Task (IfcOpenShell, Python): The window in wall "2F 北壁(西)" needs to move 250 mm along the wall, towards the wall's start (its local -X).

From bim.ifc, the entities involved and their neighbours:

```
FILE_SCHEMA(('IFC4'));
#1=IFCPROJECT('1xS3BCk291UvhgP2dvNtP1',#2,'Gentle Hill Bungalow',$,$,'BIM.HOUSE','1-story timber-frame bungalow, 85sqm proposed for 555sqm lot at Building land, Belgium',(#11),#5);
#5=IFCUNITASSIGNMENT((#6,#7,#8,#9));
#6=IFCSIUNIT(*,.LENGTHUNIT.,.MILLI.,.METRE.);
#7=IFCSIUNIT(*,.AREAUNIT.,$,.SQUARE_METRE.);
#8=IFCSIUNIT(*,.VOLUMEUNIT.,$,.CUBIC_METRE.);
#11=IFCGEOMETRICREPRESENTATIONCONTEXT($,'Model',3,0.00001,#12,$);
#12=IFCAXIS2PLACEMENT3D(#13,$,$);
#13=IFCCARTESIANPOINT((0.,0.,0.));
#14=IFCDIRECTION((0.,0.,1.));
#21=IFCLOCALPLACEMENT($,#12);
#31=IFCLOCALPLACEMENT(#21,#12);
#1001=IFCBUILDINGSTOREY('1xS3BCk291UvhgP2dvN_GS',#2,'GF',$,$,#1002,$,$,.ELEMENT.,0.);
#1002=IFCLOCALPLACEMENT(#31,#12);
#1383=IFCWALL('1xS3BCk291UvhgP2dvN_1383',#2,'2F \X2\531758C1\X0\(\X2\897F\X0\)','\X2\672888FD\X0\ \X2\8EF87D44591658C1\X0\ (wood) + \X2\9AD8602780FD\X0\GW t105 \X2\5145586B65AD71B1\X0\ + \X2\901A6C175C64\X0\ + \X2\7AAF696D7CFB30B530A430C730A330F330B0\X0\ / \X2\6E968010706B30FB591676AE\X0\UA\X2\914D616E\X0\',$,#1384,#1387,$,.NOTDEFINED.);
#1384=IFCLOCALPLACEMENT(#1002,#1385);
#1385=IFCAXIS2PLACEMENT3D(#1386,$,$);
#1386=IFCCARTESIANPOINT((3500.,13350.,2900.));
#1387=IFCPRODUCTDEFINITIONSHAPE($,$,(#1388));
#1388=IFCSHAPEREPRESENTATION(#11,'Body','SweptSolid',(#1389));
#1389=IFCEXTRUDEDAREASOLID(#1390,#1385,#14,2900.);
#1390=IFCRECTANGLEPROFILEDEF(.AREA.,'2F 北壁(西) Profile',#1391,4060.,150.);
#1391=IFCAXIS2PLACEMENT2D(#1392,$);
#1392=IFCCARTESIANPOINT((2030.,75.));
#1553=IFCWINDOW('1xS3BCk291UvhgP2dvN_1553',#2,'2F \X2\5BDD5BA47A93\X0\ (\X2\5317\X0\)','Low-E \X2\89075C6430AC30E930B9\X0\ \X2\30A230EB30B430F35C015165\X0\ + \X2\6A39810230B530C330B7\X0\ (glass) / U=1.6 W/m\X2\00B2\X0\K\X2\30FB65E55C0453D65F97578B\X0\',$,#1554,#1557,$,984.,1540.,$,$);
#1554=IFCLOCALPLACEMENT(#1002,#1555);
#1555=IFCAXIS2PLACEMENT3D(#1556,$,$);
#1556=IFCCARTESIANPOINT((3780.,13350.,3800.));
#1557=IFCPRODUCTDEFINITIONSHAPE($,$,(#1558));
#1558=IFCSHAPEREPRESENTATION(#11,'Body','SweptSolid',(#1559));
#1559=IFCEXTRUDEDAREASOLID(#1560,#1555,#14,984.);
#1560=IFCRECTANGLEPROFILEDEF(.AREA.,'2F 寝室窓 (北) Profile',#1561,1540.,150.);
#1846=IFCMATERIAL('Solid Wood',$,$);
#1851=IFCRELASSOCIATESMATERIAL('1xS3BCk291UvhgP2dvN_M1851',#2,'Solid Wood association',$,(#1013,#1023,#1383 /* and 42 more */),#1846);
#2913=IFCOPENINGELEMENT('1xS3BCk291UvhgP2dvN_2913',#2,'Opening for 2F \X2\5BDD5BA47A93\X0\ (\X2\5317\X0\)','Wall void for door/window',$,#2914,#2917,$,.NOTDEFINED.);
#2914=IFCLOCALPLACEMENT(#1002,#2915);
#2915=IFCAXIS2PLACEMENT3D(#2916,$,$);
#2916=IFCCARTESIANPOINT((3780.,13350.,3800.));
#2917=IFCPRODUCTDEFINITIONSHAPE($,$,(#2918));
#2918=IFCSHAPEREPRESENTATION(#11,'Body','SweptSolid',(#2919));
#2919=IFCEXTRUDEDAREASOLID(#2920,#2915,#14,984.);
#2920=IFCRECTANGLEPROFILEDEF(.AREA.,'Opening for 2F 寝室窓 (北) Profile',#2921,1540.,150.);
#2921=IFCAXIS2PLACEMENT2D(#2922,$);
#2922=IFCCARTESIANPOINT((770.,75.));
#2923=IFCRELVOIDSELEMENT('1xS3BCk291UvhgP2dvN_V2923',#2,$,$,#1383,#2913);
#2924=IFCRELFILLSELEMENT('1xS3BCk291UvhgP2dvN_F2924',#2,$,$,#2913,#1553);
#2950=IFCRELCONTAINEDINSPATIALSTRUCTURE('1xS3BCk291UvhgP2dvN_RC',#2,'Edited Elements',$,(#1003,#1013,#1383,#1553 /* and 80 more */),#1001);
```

```python
import ifcopenshell
import ifcopenshell.api.geometry
import ifcopenshell.util.placement
import ifcopenshell.util.unit

model = ifcopenshell.open("bim.ifc")
unit_scale = ifcopenshell.util.unit.calculate_unit_scale(model)

window = model.by_guid("1xS3BCk291UvhgP2dvN_1553")
opening = window.FillsVoids[0].RelatingOpeningElement
wall = opening.VoidsElements[0].RelatingBuildingElement

wall_matrix = ifcopenshell.util.placement.get_local_placement(wall.ObjectPlacement)
shift = wall_matrix[:3, 0] * -0.25 / unit_scale
before = ifcopenshell.util.placement.get_local_placement(window.ObjectPlacement)[:3, 3].copy()

# The window is not placed relative to its opening, so move both.
for product in (opening, window):
    matrix = ifcopenshell.util.placement.get_local_placement(product.ObjectPlacement)
    matrix[:3, 3] += shift
    ifcopenshell.api.geometry.edit_object_placement(model, product=product, matrix=matrix, is_si=False)

after = ifcopenshell.util.placement.get_local_placement(window.ObjectPlacement)[:3, 3]
print("window moved by", (after - before).round(3) + 0.0)

model.write("bim_edited.ifc")
```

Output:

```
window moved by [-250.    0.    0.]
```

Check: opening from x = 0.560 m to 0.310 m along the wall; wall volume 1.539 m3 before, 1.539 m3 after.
